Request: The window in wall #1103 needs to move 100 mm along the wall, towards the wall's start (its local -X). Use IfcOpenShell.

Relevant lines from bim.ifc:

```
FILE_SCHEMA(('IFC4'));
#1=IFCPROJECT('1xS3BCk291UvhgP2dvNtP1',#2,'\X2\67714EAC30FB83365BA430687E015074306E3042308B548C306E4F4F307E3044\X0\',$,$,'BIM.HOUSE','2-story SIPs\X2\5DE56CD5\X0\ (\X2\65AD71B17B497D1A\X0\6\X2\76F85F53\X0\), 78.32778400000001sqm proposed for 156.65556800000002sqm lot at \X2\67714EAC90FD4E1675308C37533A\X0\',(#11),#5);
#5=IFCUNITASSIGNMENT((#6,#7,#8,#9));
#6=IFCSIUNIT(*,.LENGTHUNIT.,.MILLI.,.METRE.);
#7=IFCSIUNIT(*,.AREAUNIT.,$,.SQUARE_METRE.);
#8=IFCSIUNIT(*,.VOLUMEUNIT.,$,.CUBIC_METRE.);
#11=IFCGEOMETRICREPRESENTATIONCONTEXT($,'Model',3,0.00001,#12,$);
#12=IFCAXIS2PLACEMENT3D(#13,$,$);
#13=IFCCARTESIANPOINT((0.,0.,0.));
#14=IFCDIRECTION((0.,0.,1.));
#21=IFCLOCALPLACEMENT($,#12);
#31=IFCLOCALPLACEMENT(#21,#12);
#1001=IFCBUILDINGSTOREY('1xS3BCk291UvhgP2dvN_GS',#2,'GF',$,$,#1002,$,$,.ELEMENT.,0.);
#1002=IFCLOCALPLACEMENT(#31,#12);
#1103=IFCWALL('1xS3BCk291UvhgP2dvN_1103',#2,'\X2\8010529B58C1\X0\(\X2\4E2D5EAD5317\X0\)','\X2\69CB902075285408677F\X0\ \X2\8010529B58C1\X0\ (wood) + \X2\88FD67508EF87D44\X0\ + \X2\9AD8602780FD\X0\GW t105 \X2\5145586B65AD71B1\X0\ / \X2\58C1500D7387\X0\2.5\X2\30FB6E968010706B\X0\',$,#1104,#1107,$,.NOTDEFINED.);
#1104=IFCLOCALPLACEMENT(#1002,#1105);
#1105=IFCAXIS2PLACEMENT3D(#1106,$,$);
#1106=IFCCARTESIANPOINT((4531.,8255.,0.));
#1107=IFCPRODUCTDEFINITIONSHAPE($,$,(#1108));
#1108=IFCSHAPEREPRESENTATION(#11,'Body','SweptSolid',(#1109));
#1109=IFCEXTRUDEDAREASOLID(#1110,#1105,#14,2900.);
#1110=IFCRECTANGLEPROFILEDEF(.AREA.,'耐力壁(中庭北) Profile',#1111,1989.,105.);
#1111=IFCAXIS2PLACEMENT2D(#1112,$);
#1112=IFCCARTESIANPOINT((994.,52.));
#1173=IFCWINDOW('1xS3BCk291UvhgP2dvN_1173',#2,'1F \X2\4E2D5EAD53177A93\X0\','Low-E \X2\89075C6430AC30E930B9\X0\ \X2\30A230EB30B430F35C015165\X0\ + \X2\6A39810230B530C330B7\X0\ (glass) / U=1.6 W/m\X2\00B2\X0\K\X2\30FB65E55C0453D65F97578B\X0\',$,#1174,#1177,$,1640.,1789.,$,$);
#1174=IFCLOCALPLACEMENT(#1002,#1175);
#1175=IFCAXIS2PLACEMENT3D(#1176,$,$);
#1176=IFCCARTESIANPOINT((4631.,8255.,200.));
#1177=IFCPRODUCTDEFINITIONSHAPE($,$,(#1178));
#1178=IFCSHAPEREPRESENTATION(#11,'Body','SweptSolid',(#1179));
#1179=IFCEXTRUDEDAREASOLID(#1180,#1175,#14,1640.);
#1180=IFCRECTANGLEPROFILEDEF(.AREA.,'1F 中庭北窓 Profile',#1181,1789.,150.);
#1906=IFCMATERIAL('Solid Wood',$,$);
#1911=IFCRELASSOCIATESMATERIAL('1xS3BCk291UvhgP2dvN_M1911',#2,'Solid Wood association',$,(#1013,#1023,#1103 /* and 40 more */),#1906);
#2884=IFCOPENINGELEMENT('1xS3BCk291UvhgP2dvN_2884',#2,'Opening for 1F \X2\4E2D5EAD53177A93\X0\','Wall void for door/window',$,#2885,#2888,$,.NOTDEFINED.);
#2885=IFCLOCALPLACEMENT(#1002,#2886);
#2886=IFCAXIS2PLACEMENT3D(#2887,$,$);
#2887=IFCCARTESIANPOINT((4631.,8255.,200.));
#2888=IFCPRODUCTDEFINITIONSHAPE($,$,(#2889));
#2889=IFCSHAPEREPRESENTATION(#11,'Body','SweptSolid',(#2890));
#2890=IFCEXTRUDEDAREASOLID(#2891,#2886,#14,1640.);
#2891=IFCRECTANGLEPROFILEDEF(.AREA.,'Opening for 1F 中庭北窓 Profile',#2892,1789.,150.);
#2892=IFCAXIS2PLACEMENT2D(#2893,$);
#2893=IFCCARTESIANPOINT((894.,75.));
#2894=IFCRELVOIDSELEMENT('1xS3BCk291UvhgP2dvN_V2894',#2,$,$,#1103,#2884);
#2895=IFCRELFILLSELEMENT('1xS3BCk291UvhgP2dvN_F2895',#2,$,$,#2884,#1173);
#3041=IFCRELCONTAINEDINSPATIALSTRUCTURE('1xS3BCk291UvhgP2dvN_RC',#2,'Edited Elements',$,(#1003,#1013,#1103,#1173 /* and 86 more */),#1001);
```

```python
import ifcopenshell
import ifcopenshell.api.geometry
import ifcopenshell.util.placement
import ifcopenshell.util.unit

model = ifcopenshell.open("bim.ifc")
unit_scale = ifcopenshell.util.unit.calculate_unit_scale(model)

window = model.by_guid("1xS3BCk291UvhgP2dvN_1173")
opening = window.FillsVoids[0].RelatingOpeningElement
wall = opening.VoidsElements[0].RelatingBuildingElement

wall_matrix = ifcopenshell.util.placement.get_local_placement(wall.ObjectPlacement)
shift = wall_matrix[:3, 0] * -0.1 / unit_scale
before = ifcopenshell.util.placement.get_local_placement(window.ObjectPlacement)[:3, 3].copy()

# The window is not placed relative to its opening, so move both.
for product in (opening, window):
    matrix = ifcopenshell.util.placement.get_local_placement(product.ObjectPlacement)
    matrix[:3, 3] += shift
    ifcopenshell.api.geometry.edit_object_placement(model, product=product, matrix=matrix, is_si=False)

after = ifcopenshell.util.placement.get_local_placement(window.ObjectPlacement)[:3, 3]
print("window moved by", (after - before).round(3) + 0.0)

model.write("bim_rev.ifc")
```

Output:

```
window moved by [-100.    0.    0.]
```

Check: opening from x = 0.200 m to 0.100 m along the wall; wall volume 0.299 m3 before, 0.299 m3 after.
